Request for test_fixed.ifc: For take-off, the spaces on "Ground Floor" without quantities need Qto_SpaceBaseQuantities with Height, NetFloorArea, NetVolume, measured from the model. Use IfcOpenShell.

First a look at what the model holds.

```python
import ifcopenshell
import ifcopenshell.util.element
import ifcopenshell.util.unit

model = ifcopenshell.open("test_fixed.ifc")
print(model.schema)
for unit_type in ("LENGTHUNIT", "AREAUNIT", "VOLUMEUNIT"):
    print(unit_type, ifcopenshell.util.unit.calculate_unit_scale(model, unit_type))
storey = next(s for s in model.by_type("IfcBuildingStorey") if s.Name == "Ground Floor")
spaces = [e for e in ifcopenshell.util.element.get_decomposition(storey) if e.is_a("IfcSpace")]
for e in sorted(spaces, key=lambda e: e.id()):
    print(e.id(), e.is_a(), e.Name, list(ifcopenshell.util.element.get_psets(e, qtos_only=True)), sep=" | ")
```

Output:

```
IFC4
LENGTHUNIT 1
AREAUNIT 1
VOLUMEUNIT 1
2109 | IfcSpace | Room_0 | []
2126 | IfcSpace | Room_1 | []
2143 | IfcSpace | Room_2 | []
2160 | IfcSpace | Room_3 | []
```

```python
import ifcopenshell
import ifcopenshell.api.pset
import ifcopenshell.geom
import ifcopenshell.util.element
import ifcopenshell.util.shape
import ifcopenshell.util.unit

model = ifcopenshell.open("test_fixed.ifc")
unit_scale = ifcopenshell.util.unit.calculate_unit_scale(model)
area_scale = ifcopenshell.util.unit.calculate_unit_scale(model, "AREAUNIT")
volume_scale = ifcopenshell.util.unit.calculate_unit_scale(model, "VOLUMEUNIT")
settings = ifcopenshell.geom.settings()

storey = next(s for s in model.by_type("IfcBuildingStorey") if s.Name == "Ground Floor")
spaces = [e for e in ifcopenshell.util.element.get_decomposition(storey) if e.is_a("IfcSpace")]

for e in sorted(spaces, key=lambda e: e.id()):
    if ifcopenshell.util.element.get_psets(e, qtos_only=True, should_inherit=False):
        continue
    # Geometry comes back in metres, in the element's own axes.
    shape = ifcopenshell.geom.create_shape(settings, e)
    values = {
        "Height": ifcopenshell.util.shape.get_z(shape.geometry) / unit_scale,
        "NetFloorArea": ifcopenshell.util.shape.get_footprint_area(shape.geometry) / area_scale,
        "NetVolume": ifcopenshell.util.shape.get_volume(shape.geometry) / volume_scale,
    }
    qto = ifcopenshell.api.pset.add_qto(model, product=e, name="Qto_SpaceBaseQuantities")
    ifcopenshell.api.pset.edit_qto(model, qto=qto, properties=values)
    print(e.id(), {k: round(v, 3) for k, v in values.items()})

model.write("test_fixed_rev.ifc")
```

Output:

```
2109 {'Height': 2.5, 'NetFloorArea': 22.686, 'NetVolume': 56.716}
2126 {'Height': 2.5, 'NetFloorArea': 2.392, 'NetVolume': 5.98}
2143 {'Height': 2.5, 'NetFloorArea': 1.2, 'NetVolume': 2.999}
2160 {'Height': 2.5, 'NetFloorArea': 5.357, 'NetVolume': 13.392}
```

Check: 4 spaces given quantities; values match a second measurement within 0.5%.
